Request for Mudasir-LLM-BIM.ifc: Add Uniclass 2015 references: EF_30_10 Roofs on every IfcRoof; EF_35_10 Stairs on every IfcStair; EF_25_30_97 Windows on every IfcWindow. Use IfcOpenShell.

First a look at what the model holds.

```python
import ifcopenshell

model = ifcopenshell.open("Mudasir-LLM-BIM.ifc")
print(model.schema)
print("classifications:", [c.Name for c in model.by_type("IfcClassification")])
for ifc_class in ("IfcDoor", "IfcRoof", "IfcStair", "IfcWall", "IfcWindow"):
    print(ifc_class, len(model.by_type(ifc_class)))
```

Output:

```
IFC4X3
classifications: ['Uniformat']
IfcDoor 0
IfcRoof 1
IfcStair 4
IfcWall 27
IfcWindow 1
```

```python
import ifcopenshell
import ifcopenshell.api.classification

model = ifcopenshell.open("Mudasir-LLM-BIM.ifc")

system = ifcopenshell.api.classification.add_classification(model, classification="Uniclass 2015")

codes = {
    "IfcRoof": ("EF_30_10", "Roofs"),
    "IfcStair": ("EF_35_10", "Stairs"),
    "IfcWindow": ("EF_25_30_97", "Windows"),
}
for ifc_class, (code, name) in codes.items():
    products = model.by_type(ifc_class)
    ifcopenshell.api.classification.add_reference(
        model, products=products, classification=system, identification=code, name=name
    )
    print(code, len(products))

model.write("Mudasir-LLM-BIM_edited.ifc")
```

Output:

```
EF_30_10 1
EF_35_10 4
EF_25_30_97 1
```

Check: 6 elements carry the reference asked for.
